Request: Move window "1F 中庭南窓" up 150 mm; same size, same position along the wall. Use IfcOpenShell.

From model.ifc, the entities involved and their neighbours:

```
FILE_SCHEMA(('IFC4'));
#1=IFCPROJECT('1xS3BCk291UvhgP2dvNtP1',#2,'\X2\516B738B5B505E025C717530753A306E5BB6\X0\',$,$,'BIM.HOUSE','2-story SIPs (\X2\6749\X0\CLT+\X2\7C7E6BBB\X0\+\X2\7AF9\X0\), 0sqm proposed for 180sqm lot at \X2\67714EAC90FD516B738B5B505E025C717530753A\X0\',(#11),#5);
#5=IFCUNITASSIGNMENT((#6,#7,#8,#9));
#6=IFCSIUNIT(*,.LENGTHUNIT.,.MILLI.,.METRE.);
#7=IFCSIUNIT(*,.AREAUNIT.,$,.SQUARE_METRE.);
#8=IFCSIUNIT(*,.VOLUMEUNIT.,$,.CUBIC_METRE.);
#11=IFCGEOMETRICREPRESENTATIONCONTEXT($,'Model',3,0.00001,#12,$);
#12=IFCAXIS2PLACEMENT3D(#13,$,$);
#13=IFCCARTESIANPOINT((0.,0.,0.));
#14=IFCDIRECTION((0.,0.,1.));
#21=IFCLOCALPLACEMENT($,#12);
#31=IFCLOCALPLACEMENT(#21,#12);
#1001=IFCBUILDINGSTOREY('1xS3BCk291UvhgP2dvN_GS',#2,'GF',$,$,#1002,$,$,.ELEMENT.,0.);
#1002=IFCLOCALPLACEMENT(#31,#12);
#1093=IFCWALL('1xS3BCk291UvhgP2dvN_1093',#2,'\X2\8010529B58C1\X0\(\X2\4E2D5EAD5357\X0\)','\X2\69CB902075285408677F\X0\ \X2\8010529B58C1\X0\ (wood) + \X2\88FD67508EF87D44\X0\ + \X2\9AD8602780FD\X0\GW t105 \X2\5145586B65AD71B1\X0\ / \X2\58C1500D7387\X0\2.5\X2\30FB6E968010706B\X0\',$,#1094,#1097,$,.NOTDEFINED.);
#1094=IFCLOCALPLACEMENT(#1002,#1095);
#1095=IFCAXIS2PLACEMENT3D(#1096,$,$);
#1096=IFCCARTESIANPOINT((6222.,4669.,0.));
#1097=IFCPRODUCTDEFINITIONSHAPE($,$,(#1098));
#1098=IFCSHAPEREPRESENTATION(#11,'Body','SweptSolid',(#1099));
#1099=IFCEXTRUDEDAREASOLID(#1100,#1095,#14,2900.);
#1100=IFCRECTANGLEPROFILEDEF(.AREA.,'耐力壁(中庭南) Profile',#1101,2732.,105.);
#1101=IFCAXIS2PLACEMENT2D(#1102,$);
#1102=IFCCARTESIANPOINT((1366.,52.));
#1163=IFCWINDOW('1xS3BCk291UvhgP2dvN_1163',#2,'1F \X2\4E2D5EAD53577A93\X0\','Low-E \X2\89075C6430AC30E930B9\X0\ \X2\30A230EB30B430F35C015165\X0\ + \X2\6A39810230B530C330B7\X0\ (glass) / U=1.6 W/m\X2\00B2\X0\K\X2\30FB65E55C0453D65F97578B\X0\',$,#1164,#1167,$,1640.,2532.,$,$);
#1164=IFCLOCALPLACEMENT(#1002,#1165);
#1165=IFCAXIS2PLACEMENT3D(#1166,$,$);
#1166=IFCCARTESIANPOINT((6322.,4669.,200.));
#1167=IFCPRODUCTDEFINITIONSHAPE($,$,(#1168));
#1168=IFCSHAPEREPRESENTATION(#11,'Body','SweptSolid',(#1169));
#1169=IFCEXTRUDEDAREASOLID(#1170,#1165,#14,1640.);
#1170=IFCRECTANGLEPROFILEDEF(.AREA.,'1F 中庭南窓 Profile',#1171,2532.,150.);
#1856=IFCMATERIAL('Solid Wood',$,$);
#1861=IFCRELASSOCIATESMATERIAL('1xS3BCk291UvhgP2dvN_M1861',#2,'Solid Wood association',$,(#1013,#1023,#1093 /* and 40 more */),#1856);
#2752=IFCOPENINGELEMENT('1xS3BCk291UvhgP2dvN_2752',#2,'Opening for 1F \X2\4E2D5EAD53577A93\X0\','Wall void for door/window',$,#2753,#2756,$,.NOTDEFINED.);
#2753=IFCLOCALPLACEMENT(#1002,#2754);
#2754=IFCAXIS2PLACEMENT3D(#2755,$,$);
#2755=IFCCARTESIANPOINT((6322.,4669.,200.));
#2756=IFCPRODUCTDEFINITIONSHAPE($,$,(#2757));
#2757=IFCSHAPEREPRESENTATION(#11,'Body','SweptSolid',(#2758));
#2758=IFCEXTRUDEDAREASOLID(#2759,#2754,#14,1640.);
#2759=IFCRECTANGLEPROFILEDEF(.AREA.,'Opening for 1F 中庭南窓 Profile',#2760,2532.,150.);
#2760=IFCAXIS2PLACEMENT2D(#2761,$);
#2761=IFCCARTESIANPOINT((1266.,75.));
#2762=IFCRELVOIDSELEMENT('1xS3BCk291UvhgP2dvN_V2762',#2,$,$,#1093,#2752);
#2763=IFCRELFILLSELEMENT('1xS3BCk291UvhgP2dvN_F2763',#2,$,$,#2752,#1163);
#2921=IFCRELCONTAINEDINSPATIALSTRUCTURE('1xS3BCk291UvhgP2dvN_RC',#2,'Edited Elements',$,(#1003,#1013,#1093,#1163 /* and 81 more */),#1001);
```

```python
import numpy as np
import ifcopenshell
import ifcopenshell.api.geometry
import ifcopenshell.util.placement
import ifcopenshell.util.unit

model = ifcopenshell.open("model.ifc")
unit_scale = ifcopenshell.util.unit.calculate_unit_scale(model)

window = model.by_guid("1xS3BCk291UvhgP2dvN_1163")
opening = window.FillsVoids[0].RelatingOpeningElement
dz = 150.0

shift = np.array([0.0, 0.0, dz])
# The window is not placed relative to its opening, so move both.
for product in (opening, window):
    matrix = ifcopenshell.util.placement.get_local_placement(product.ObjectPlacement)
    matrix[:3, 3] += shift
    ifcopenshell.api.geometry.edit_object_placement(model, product=product, matrix=matrix, is_si=False)

print(f"moved by {dz * unit_scale:+.3f} m")

model.write("model_edited.ifc")
```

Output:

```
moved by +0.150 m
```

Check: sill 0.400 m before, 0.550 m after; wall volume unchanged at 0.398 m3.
